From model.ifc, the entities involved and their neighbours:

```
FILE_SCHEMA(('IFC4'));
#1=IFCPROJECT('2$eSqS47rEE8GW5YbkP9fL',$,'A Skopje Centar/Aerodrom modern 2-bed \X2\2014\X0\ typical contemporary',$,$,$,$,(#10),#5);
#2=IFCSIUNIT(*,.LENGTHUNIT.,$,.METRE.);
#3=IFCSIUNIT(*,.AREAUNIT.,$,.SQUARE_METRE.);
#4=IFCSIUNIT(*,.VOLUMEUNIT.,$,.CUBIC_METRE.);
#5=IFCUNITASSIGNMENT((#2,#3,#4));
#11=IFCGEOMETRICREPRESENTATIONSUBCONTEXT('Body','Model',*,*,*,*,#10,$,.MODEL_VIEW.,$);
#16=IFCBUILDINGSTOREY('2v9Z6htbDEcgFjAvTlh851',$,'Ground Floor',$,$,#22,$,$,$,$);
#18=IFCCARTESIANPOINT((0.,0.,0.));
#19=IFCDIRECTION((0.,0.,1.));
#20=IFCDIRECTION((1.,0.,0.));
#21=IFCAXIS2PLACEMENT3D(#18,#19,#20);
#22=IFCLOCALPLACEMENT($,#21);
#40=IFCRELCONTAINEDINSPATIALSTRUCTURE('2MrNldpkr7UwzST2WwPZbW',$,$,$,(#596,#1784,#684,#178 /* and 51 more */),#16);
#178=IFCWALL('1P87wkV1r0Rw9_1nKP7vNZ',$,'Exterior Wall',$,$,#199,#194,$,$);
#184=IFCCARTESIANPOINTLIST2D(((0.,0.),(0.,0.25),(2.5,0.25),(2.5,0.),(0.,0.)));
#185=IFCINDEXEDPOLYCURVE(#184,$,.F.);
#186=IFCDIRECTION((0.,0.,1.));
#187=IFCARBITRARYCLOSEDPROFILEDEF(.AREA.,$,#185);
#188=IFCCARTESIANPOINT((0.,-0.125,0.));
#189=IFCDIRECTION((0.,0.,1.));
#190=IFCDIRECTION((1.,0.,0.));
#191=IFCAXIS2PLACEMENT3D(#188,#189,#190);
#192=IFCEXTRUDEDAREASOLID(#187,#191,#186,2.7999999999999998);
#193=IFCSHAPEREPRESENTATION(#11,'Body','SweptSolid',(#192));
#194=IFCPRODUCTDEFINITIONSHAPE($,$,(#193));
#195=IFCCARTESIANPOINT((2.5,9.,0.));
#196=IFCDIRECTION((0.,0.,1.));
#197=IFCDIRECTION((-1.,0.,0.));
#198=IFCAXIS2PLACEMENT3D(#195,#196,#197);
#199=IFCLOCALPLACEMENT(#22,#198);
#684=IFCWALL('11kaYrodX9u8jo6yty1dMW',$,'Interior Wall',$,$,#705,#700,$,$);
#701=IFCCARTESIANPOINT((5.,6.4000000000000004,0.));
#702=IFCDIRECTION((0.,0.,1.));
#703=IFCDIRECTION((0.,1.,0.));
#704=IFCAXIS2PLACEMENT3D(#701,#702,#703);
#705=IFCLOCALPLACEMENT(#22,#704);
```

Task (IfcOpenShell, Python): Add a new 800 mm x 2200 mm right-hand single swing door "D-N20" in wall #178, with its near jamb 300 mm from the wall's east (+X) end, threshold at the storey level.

```python
import numpy as np
import ifcopenshell
import ifcopenshell.api.feature
import ifcopenshell.api.geometry
import ifcopenshell.api.root
import ifcopenshell.api.spatial
import ifcopenshell.geom
import ifcopenshell.util.element
import ifcopenshell.util.placement
import ifcopenshell.util.representation
import ifcopenshell.util.shape
import ifcopenshell.util.unit

model = ifcopenshell.open("model.ifc")
unit_scale = ifcopenshell.util.unit.calculate_unit_scale(model)
settings = ifcopenshell.geom.settings()


def volume(element):
    """Net volume in cubic metres, openings subtracted."""
    shape = ifcopenshell.geom.create_shape(settings, element)
    return ifcopenshell.util.shape.get_volume(shape.geometry)


wall = model.by_guid("1P87wkV1r0Rw9_1nKP7vNZ")
storey = ifcopenshell.util.element.get_container(wall, ifc_class="IfcBuildingStorey")
context = ifcopenshell.util.representation.get_context(model, "Model", "Body", "MODEL_VIEW")
before = volume(wall)

width, height, from_end, sill = 0.8, 2.2, 0.3, 0.0  # metres

# The wall runs along its own X axis, and the end named is its -X end.
wall_shape = ifcopenshell.geom.create_shape(settings, wall)
x, y, z = ifcopenshell.util.shape.get_vertices(wall_shape.geometry).T
start = x.min() + from_end
face, thickness = float(y.min()), float(y.max() - y.min())
wall_matrix = ifcopenshell.util.placement.get_local_placement(wall.ObjectPlacement)
level = ifcopenshell.util.placement.get_local_placement(storey.ObjectPlacement)[2, 3]


def in_wall(x, y):
    """Placement at x, y metres in the wall's axes, at sill height."""
    matrix = wall_matrix.copy()
    matrix[:, 3] = wall_matrix @ np.array([x / unit_scale, y / unit_scale, 0.0, 1.0])
    matrix[2, 3] = level + sill / unit_scale
    return matrix


# Opening: a box that overshoots both wall faces by 50 mm.
opening = ifcopenshell.api.root.create_entity(model, ifc_class="IfcOpeningElement", predefined_type="OPENING")
box = ifcopenshell.api.geometry.add_wall_representation(
    model, context=context, length=width, height=height, thickness=thickness + 0.1
)
ifcopenshell.api.geometry.assign_representation(model, product=opening, representation=box)
ifcopenshell.api.geometry.edit_object_placement(model, product=opening, matrix=in_wall(start, face - 0.05), is_si=False)
ifcopenshell.api.feature.add_feature(model, feature=opening, element=wall)

door = ifcopenshell.api.root.create_entity(model, ifc_class="IfcDoor", name="D-N20", predefined_type="DOOR")
door.OverallWidth, door.OverallHeight = width / unit_scale, height / unit_scale
door.OperationType = "SINGLE_SWING_RIGHT"
body = ifcopenshell.api.geometry.add_door_representation(
    model,
    context=context,
    overall_width=door.OverallWidth,
    overall_height=door.OverallHeight,
    operation_type="SINGLE_SWING_RIGHT",
    lining_properties={"LiningDepth": thickness / unit_scale, "ThresholdDepth": thickness / unit_scale},
)
ifcopenshell.api.geometry.assign_representation(model, product=door, representation=body)
ifcopenshell.api.spatial.assign_container(model, products=[door], relating_structure=storey)
ifcopenshell.api.feature.add_filling(model, opening=opening, element=door)

# The lining spans the wall, so the door starts at the wall face.
ifcopenshell.api.geometry.edit_object_placement(model, product=door, matrix=in_wall(start, face), is_si=False)

after = volume(wall)

print(f"wall volume {before:.3f} -> {after:.3f} m3")

model.write("model_v2.ifc")
```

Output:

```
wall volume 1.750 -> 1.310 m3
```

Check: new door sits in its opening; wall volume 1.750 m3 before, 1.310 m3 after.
